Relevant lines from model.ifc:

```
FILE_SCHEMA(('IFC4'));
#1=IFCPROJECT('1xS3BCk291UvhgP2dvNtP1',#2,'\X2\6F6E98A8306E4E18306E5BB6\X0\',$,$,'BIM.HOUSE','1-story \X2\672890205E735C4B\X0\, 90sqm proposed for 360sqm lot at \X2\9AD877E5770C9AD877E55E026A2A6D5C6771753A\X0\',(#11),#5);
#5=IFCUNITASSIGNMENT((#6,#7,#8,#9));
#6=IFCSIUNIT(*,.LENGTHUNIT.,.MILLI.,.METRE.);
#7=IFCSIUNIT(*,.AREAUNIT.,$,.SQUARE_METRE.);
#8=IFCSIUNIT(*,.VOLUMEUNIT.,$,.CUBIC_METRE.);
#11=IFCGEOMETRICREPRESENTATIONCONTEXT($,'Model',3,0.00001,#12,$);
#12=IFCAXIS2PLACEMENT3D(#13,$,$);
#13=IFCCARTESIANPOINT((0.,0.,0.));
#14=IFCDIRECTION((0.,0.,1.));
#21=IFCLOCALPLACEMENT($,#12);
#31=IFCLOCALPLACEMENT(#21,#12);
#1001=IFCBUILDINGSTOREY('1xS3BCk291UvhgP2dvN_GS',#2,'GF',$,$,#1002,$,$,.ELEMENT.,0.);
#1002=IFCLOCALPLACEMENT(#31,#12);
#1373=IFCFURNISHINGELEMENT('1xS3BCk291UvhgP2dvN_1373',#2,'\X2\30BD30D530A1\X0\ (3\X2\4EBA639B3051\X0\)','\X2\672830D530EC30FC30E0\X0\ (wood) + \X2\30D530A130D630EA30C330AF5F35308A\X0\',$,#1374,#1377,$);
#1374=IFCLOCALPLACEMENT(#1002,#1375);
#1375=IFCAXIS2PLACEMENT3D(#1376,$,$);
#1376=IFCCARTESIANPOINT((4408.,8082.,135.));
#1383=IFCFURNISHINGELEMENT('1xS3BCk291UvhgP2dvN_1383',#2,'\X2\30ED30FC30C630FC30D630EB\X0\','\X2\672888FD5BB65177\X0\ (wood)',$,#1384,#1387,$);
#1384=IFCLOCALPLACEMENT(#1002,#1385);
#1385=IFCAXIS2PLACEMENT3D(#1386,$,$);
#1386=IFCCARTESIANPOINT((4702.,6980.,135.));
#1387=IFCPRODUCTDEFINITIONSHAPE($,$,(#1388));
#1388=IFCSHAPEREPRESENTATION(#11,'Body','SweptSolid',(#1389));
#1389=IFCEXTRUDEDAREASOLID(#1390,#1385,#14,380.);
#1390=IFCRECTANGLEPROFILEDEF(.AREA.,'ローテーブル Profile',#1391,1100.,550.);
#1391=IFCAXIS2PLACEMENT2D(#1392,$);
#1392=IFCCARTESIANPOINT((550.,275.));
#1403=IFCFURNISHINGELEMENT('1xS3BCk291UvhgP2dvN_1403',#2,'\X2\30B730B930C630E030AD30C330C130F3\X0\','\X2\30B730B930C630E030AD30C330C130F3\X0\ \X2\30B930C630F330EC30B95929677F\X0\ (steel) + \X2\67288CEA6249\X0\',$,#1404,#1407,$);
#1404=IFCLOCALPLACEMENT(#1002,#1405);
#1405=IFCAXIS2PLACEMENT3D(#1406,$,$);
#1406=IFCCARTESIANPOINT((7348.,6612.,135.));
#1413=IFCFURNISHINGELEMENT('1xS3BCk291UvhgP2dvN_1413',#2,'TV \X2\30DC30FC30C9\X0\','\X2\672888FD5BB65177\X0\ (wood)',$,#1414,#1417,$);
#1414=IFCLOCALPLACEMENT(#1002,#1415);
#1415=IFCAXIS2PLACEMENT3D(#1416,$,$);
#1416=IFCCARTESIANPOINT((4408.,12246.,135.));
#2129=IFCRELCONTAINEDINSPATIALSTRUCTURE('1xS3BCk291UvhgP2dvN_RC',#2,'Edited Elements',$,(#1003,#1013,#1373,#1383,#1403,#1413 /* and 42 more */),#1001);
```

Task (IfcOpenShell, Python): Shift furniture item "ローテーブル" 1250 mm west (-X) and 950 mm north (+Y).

```python
import ifcopenshell
import ifcopenshell.api.geometry
import ifcopenshell.util.placement
import ifcopenshell.util.unit

model = ifcopenshell.open("model.ifc")
unit_scale = ifcopenshell.util.unit.calculate_unit_scale(model)

item = model.by_id(1383)
matrix = ifcopenshell.util.placement.get_local_placement(item.ObjectPlacement)
matrix[0, 3] -= 1.25 / unit_scale
matrix[1, 3] += 0.95 / unit_scale
ifcopenshell.api.geometry.edit_object_placement(model, product=item, matrix=matrix, is_si=False)

print(ifcopenshell.util.placement.get_local_placement(item.ObjectPlacement).round(3) + 0.0)

model.write("model_updated.ifc")
```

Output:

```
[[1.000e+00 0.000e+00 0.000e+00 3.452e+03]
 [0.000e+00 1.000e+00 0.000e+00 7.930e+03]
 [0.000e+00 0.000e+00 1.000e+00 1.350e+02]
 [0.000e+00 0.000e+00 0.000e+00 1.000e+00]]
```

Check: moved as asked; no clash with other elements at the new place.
